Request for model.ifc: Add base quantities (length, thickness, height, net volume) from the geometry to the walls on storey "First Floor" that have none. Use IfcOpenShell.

First a look at what the model holds.

```python
import ifcopenshell
import ifcopenshell.util.element
import ifcopenshell.util.unit

model = ifcopenshell.open("model.ifc")
print(model.schema)
for unit_type in ("LENGTHUNIT", "AREAUNIT", "VOLUMEUNIT"):
    print(unit_type, ifcopenshell.util.unit.calculate_unit_scale(model, unit_type))
storey = next(s for s in model.by_type("IfcBuildingStorey") if s.Name == "First Floor")
walls = [e for e in ifcopenshell.util.element.get_decomposition(storey) if e.is_a("IfcWall")]
for e in sorted(walls, key=lambda e: e.id()):
    print(e.id(), e.is_a(), e.Name, list(ifcopenshell.util.element.get_psets(e, qtos_only=True)), sep=" | ")
```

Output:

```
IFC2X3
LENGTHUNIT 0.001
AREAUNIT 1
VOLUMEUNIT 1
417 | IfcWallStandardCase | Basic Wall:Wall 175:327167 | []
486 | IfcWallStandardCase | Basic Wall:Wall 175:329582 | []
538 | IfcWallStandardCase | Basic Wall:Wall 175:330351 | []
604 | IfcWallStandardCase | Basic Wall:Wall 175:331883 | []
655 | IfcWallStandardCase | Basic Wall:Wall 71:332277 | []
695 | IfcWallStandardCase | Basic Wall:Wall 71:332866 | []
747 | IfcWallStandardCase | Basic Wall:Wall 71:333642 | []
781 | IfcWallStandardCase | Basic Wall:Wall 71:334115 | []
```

```python
import ifcopenshell
import ifcopenshell.api.pset
import ifcopenshell.geom
import ifcopenshell.util.element
import ifcopenshell.util.shape
import ifcopenshell.util.unit

model = ifcopenshell.open("model.ifc")
unit_scale = ifcopenshell.util.unit.calculate_unit_scale(model)
volume_scale = ifcopenshell.util.unit.calculate_unit_scale(model, "VOLUMEUNIT")
settings = ifcopenshell.geom.settings()

storey = next(s for s in model.by_type("IfcBuildingStorey") if s.Name == "First Floor")
walls = [e for e in ifcopenshell.util.element.get_decomposition(storey) if e.is_a("IfcWall")]

for e in sorted(walls, key=lambda e: e.id()):
    if ifcopenshell.util.element.get_psets(e, qtos_only=True, should_inherit=False):
        continue
    # Geometry comes back in metres, in the element's own axes.
    shape = ifcopenshell.geom.create_shape(settings, e)
    values = {
        "Length": ifcopenshell.util.shape.get_x(shape.geometry) / unit_scale,
        "Width": ifcopenshell.util.shape.get_y(shape.geometry) / unit_scale,
        "Height": ifcopenshell.util.shape.get_z(shape.geometry) / unit_scale,
        "NetVolume": ifcopenshell.util.shape.get_volume(shape.geometry) / volume_scale,
    }
    qto = ifcopenshell.api.pset.add_qto(model, product=e, name="BaseQuantities")
    ifcopenshell.api.pset.edit_qto(model, qto=qto, properties=values)
    print(e.id(), {k: round(v, 3) for k, v in values.items()})

model.write("model-out.ifc")
```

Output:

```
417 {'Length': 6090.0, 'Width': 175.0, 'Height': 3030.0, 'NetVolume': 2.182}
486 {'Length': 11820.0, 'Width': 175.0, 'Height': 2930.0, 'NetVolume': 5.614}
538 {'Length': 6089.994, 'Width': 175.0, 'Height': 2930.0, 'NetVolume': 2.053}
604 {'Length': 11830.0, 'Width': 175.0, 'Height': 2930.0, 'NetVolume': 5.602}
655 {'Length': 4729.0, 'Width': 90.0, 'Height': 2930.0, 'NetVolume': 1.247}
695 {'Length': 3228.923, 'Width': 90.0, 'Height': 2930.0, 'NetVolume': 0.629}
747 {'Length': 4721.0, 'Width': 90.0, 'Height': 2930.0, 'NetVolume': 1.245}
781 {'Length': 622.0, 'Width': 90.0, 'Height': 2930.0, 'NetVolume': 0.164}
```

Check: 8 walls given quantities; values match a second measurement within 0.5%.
